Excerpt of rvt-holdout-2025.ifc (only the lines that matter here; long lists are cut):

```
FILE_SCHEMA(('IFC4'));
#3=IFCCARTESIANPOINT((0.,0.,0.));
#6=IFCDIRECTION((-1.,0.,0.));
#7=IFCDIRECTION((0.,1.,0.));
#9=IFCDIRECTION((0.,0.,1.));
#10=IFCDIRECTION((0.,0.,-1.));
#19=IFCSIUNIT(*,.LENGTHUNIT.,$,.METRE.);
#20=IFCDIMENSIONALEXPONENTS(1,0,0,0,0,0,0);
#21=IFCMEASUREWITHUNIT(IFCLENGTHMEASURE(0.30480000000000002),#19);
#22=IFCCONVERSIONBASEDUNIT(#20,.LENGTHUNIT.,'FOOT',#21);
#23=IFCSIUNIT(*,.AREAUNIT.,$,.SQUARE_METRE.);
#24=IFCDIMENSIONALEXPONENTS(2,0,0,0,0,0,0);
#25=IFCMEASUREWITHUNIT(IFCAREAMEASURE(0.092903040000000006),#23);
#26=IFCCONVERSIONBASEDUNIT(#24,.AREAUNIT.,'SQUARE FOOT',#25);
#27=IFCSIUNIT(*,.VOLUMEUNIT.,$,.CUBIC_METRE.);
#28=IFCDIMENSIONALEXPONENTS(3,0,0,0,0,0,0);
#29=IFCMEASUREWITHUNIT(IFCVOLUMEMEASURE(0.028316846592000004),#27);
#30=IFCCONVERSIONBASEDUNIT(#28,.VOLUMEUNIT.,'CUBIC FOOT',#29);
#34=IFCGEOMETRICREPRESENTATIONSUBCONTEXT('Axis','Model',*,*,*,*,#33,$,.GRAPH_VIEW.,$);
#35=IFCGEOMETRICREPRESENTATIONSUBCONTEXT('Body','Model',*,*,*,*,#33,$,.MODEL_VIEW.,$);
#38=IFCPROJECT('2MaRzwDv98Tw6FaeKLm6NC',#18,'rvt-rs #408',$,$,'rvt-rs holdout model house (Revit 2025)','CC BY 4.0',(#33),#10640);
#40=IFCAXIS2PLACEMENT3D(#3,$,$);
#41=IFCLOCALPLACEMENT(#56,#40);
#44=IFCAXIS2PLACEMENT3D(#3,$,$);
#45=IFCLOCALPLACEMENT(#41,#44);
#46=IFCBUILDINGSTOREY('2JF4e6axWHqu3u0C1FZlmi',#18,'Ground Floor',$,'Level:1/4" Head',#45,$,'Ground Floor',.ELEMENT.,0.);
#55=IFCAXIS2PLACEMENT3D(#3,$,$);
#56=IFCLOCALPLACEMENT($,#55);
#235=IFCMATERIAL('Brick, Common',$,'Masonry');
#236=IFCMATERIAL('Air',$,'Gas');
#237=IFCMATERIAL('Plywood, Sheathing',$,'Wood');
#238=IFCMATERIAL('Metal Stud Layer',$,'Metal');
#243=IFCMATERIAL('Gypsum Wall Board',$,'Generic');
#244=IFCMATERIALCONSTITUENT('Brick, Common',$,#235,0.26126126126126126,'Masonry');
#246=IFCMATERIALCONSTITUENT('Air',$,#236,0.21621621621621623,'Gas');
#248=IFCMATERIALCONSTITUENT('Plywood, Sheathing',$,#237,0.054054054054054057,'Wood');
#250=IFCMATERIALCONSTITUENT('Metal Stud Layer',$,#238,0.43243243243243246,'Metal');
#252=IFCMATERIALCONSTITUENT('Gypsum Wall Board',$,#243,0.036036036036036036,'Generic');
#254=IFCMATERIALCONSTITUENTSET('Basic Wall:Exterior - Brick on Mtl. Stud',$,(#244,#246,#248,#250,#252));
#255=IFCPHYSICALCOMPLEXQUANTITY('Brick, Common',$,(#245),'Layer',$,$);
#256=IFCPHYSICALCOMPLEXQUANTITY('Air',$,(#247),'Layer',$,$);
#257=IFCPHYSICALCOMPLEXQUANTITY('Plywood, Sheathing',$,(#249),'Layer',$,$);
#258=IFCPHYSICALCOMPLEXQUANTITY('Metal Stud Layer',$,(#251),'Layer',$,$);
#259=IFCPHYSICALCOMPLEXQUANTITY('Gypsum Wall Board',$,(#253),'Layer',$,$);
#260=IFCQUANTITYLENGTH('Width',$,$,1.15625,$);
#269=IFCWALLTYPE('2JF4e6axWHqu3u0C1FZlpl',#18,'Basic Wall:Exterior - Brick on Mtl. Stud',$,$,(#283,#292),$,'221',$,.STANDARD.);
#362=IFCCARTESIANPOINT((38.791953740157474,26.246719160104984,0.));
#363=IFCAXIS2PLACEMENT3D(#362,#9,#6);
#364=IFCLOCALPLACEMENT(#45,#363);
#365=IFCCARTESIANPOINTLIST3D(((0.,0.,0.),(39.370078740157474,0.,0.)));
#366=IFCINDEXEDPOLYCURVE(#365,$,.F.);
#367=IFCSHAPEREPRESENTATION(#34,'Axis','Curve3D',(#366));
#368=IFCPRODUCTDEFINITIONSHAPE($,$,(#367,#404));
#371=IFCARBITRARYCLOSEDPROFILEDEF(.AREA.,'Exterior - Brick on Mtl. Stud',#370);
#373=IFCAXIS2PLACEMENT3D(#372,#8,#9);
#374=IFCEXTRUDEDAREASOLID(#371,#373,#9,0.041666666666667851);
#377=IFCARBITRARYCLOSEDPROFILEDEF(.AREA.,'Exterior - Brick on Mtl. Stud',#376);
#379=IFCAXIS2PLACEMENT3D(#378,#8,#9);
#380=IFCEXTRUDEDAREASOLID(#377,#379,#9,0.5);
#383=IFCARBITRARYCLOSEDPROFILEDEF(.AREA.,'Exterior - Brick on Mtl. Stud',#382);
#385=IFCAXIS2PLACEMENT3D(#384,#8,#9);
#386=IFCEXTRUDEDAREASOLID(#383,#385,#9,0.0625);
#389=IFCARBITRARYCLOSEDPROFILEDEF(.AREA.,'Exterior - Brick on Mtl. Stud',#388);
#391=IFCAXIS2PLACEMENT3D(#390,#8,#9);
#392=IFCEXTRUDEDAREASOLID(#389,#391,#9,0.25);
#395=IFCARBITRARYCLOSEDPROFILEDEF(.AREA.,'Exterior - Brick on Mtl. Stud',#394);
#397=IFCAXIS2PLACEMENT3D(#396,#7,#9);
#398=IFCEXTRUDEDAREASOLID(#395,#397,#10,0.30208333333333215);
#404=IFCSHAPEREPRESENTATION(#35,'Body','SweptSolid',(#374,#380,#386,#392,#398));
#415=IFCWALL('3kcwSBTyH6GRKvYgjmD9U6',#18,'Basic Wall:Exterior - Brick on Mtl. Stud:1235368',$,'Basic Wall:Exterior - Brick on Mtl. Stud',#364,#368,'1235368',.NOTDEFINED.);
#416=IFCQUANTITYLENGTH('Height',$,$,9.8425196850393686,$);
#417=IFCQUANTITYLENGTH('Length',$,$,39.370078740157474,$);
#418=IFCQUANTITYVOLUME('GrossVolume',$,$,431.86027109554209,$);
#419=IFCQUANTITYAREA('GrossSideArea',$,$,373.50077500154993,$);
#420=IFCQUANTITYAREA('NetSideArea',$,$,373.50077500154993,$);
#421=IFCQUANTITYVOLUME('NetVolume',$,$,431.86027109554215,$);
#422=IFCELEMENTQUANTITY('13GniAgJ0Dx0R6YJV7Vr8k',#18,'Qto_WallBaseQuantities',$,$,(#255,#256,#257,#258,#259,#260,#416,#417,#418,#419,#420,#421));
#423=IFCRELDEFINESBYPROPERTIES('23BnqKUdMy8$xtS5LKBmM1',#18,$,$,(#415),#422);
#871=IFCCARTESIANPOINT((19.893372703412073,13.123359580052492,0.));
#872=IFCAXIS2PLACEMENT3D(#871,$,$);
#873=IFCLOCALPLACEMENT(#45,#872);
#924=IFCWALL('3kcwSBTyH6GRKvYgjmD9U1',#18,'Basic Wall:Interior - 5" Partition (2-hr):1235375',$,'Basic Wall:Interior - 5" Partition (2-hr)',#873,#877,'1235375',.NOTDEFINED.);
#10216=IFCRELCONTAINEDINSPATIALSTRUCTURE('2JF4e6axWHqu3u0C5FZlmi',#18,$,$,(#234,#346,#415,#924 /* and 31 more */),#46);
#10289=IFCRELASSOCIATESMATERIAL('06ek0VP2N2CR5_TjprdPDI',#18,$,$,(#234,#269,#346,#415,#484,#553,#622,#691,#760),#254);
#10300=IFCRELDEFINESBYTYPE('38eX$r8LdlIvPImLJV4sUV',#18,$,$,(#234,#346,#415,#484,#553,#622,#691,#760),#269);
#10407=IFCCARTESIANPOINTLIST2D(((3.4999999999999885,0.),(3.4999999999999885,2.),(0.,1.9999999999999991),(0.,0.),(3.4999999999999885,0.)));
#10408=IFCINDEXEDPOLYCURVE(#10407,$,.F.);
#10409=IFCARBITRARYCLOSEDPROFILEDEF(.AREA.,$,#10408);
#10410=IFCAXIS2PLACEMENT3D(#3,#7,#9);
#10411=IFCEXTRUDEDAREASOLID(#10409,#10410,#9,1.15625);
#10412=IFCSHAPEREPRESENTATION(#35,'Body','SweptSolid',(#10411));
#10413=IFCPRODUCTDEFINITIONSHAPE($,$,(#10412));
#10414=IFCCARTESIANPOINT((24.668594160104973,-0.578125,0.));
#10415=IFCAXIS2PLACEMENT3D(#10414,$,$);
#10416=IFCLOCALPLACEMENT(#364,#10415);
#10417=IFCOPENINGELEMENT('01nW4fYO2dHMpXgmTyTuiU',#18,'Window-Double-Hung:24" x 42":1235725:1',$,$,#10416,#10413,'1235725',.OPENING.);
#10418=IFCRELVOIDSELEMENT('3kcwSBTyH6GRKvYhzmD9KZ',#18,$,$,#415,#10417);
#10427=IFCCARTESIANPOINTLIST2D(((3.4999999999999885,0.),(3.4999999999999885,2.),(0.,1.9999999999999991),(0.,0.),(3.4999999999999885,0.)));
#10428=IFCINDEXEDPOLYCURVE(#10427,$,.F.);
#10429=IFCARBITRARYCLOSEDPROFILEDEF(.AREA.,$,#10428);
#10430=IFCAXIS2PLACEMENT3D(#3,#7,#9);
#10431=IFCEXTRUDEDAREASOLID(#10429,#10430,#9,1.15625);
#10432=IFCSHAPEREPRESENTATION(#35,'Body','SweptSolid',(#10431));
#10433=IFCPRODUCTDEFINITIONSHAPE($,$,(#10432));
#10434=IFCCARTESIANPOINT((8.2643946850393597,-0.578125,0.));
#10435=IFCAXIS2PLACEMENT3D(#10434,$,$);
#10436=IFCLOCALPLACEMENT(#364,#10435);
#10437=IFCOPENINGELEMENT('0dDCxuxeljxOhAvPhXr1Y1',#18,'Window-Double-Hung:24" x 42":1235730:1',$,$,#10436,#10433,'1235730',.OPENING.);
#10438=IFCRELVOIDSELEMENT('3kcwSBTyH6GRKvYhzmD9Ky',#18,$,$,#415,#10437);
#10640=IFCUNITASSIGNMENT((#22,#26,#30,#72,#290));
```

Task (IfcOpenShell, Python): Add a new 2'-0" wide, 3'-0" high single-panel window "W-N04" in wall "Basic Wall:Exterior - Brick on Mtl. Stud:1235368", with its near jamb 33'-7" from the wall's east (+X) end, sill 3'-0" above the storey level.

```python
import numpy as np
import ifcopenshell
import ifcopenshell.api.feature
import ifcopenshell.api.geometry
import ifcopenshell.api.pset
import ifcopenshell.api.root
import ifcopenshell.api.spatial
import ifcopenshell.geom
import ifcopenshell.util.element
import ifcopenshell.util.placement
import ifcopenshell.util.representation
import ifcopenshell.util.shape
import ifcopenshell.util.unit

model = ifcopenshell.open("rvt-holdout-2025.ifc")
unit_scale = ifcopenshell.util.unit.calculate_unit_scale(model)
area_scale = ifcopenshell.util.unit.calculate_unit_scale(model, "AREAUNIT")
volume_scale = ifcopenshell.util.unit.calculate_unit_scale(model, "VOLUMEUNIT")
settings = ifcopenshell.geom.settings()


def volume(element):
    """Net volume in cubic metres, openings subtracted."""
    shape = ifcopenshell.geom.create_shape(settings, element)
    return ifcopenshell.util.shape.get_volume(shape.geometry)


wall = model.by_id(415)
storey = ifcopenshell.util.element.get_container(wall, ifc_class="IfcBuildingStorey")
context = ifcopenshell.util.representation.get_context(model, "Model", "Body", "MODEL_VIEW")
before = volume(wall)

width, height, from_end, sill = 0.6096, 0.9144, 10.2362, 0.9144  # metres

# The wall runs along its own X axis, and the end named is its -X end.
wall_shape = ifcopenshell.geom.create_shape(settings, wall)
x, y, z = ifcopenshell.util.shape.get_vertices(wall_shape.geometry).T
start = x.min() + from_end
face, thickness = float(y.min()), float(y.max() - y.min())
wall_matrix = ifcopenshell.util.placement.get_local_placement(wall.ObjectPlacement)
level = ifcopenshell.util.placement.get_local_placement(storey.ObjectPlacement)[2, 3]


def in_wall(x, y):
    """Placement at x, y metres in the wall's axes, at sill height."""
    matrix = wall_matrix.copy()
    matrix[:, 3] = wall_matrix @ np.array([x / unit_scale, y / unit_scale, 0.0, 1.0])
    matrix[2, 3] = level + sill / unit_scale
    return matrix


# Opening: a box that overshoots both wall faces by 50 mm.
opening = ifcopenshell.api.root.create_entity(model, ifc_class="IfcOpeningElement", predefined_type="OPENING")
box = ifcopenshell.api.geometry.add_wall_representation(
    model, context=context, length=width, height=height, thickness=thickness + 0.1
)
ifcopenshell.api.geometry.assign_representation(model, product=opening, representation=box)
ifcopenshell.api.geometry.edit_object_placement(model, product=opening, matrix=in_wall(start, face - 0.05), is_si=False)
ifcopenshell.api.feature.add_feature(model, feature=opening, element=wall)

window = ifcopenshell.api.root.create_entity(model, ifc_class="IfcWindow", name="W-N04", predefined_type="WINDOW")
window.OverallWidth, window.OverallHeight = width / unit_scale, height / unit_scale
window.PartitioningType = "SINGLE_PANEL"
body = ifcopenshell.api.geometry.add_window_representation(
    model,
    context=context,
    overall_width=window.OverallWidth,
    overall_height=window.OverallHeight,
    partition_type="SINGLE_PANEL",
)
ifcopenshell.api.geometry.assign_representation(model, product=window, representation=body)
ifcopenshell.api.spatial.assign_container(model, products=[window], relating_structure=storey)
ifcopenshell.api.feature.add_filling(model, opening=opening, element=window)

# Centre the window in the wall's thickness.
ifcopenshell.api.geometry.edit_object_placement(model, product=window, matrix=in_wall(start, face), is_si=False)
window_shape = ifcopenshell.geom.create_shape(settings, window)
depth = ifcopenshell.util.shape.get_vertices(window_shape.geometry)[:, 1]
offset = face + thickness / 2 - (depth.min() + depth.max()) / 2
ifcopenshell.api.geometry.edit_object_placement(model, product=window, matrix=in_wall(start, offset), is_si=False)

after = volume(wall)

# Update the wall's stored quantities.
qto = model.by_id(ifcopenshell.util.element.get_pset(wall, "Qto_WallBaseQuantities", should_inherit=False)["id"])
ifcopenshell.api.pset.edit_qto(model, qto=qto, properties={
    "NetSideArea": after / thickness / area_scale,
    "NetVolume": after / volume_scale,
})

print(f"wall volume {before:.3f} -> {after:.3f} m3")

model.write("rvt-holdout-2025-out.ifc")
```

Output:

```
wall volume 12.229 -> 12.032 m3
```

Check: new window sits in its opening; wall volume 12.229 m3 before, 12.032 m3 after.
